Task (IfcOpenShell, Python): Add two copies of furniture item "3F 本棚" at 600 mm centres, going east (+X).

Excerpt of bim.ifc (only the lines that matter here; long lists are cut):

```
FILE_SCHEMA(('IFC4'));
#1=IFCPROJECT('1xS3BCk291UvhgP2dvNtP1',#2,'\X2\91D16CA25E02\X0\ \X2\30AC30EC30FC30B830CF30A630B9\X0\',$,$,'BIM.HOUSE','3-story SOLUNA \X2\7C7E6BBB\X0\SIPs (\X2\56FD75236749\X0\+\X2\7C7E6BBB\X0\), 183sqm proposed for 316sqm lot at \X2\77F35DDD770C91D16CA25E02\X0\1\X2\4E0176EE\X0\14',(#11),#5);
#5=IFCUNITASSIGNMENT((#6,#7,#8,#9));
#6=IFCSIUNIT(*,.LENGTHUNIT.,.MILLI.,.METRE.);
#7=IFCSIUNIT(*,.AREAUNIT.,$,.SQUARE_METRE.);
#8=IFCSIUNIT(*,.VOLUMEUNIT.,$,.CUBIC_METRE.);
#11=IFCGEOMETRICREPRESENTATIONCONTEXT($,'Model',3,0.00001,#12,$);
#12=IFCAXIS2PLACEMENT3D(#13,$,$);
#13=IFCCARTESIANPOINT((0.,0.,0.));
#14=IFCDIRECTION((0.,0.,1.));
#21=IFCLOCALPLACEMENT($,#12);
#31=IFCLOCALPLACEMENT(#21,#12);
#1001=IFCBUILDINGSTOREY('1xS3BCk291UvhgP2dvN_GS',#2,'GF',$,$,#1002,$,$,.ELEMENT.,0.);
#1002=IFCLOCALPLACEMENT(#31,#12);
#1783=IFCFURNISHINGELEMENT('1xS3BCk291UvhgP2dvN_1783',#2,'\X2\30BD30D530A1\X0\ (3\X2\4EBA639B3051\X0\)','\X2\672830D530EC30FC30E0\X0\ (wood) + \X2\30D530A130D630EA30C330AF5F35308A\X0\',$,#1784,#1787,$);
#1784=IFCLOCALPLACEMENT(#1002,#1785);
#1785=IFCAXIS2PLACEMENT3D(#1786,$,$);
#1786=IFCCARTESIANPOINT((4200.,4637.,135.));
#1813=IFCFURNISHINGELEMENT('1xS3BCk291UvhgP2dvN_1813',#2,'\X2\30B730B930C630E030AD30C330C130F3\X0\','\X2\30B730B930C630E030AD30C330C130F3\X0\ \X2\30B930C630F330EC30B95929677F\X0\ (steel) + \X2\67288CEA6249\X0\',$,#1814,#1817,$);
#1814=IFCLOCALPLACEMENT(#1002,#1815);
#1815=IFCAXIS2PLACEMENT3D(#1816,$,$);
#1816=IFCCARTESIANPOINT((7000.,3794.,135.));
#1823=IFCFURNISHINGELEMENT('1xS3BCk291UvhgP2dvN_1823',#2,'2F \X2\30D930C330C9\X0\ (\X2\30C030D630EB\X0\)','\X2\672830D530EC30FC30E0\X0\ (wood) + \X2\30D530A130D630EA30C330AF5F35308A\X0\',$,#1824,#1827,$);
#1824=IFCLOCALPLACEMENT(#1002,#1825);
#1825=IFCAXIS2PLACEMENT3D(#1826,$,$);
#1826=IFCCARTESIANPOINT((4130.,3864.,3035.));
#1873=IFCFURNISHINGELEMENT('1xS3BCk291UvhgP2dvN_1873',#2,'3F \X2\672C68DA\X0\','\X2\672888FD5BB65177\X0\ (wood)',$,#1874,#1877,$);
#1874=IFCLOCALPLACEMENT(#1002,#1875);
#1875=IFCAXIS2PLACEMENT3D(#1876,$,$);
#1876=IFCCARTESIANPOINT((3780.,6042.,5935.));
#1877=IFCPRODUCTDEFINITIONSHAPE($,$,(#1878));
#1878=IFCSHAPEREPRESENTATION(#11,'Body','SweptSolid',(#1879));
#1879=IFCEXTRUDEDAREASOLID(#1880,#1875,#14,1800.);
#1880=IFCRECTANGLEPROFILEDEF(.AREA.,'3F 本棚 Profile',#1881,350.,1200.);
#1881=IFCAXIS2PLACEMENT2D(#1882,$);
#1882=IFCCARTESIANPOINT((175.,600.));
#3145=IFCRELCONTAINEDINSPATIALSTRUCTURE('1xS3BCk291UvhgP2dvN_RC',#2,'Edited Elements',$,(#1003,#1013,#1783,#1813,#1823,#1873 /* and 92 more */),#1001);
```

```python
import numpy as np
import ifcopenshell
import ifcopenshell.api.geometry
import ifcopenshell.api.root
import ifcopenshell.util.element
import ifcopenshell.util.placement

model = ifcopenshell.open("bim.ifc")


def reuse_history(source, copy):
    """copy_class also copies each property set's owner history, people and application; keep the originals."""
    for rel in copy.IsDefinedBy:
        if rel.is_a("IfcRelDefinesByProperties") and (history := rel.RelatingPropertyDefinition.OwnerHistory):
            rel.RelatingPropertyDefinition.OwnerHistory = source.OwnerHistory
            ifcopenshell.util.element.remove_deep2(model, history)


source = model.by_guid("1xS3BCk291UvhgP2dvN_1873")
base = ifcopenshell.util.placement.get_local_placement(source.ObjectPlacement)
step = np.array([1.0, 0.0, 0.0]) * 600.0

for i in range(1, 3):
    copy = ifcopenshell.api.root.copy_class(model, product=source)
    copy.Representation = ifcopenshell.util.element.copy_deep(
        model, source.Representation, exclude=["IfcGeometricRepresentationContext", "IfcRepresentationMap"]
    )
    reuse_history(source, copy)
    matrix = base.copy()
    matrix[:3, 3] += i * step
    print("added at", matrix[:3, 3].round(3) + 0.0)
    ifcopenshell.api.geometry.edit_object_placement(model, product=copy, matrix=matrix, is_si=False)

model.write("bim_updated.ifc")
```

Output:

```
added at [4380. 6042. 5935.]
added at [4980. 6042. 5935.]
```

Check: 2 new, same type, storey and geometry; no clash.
